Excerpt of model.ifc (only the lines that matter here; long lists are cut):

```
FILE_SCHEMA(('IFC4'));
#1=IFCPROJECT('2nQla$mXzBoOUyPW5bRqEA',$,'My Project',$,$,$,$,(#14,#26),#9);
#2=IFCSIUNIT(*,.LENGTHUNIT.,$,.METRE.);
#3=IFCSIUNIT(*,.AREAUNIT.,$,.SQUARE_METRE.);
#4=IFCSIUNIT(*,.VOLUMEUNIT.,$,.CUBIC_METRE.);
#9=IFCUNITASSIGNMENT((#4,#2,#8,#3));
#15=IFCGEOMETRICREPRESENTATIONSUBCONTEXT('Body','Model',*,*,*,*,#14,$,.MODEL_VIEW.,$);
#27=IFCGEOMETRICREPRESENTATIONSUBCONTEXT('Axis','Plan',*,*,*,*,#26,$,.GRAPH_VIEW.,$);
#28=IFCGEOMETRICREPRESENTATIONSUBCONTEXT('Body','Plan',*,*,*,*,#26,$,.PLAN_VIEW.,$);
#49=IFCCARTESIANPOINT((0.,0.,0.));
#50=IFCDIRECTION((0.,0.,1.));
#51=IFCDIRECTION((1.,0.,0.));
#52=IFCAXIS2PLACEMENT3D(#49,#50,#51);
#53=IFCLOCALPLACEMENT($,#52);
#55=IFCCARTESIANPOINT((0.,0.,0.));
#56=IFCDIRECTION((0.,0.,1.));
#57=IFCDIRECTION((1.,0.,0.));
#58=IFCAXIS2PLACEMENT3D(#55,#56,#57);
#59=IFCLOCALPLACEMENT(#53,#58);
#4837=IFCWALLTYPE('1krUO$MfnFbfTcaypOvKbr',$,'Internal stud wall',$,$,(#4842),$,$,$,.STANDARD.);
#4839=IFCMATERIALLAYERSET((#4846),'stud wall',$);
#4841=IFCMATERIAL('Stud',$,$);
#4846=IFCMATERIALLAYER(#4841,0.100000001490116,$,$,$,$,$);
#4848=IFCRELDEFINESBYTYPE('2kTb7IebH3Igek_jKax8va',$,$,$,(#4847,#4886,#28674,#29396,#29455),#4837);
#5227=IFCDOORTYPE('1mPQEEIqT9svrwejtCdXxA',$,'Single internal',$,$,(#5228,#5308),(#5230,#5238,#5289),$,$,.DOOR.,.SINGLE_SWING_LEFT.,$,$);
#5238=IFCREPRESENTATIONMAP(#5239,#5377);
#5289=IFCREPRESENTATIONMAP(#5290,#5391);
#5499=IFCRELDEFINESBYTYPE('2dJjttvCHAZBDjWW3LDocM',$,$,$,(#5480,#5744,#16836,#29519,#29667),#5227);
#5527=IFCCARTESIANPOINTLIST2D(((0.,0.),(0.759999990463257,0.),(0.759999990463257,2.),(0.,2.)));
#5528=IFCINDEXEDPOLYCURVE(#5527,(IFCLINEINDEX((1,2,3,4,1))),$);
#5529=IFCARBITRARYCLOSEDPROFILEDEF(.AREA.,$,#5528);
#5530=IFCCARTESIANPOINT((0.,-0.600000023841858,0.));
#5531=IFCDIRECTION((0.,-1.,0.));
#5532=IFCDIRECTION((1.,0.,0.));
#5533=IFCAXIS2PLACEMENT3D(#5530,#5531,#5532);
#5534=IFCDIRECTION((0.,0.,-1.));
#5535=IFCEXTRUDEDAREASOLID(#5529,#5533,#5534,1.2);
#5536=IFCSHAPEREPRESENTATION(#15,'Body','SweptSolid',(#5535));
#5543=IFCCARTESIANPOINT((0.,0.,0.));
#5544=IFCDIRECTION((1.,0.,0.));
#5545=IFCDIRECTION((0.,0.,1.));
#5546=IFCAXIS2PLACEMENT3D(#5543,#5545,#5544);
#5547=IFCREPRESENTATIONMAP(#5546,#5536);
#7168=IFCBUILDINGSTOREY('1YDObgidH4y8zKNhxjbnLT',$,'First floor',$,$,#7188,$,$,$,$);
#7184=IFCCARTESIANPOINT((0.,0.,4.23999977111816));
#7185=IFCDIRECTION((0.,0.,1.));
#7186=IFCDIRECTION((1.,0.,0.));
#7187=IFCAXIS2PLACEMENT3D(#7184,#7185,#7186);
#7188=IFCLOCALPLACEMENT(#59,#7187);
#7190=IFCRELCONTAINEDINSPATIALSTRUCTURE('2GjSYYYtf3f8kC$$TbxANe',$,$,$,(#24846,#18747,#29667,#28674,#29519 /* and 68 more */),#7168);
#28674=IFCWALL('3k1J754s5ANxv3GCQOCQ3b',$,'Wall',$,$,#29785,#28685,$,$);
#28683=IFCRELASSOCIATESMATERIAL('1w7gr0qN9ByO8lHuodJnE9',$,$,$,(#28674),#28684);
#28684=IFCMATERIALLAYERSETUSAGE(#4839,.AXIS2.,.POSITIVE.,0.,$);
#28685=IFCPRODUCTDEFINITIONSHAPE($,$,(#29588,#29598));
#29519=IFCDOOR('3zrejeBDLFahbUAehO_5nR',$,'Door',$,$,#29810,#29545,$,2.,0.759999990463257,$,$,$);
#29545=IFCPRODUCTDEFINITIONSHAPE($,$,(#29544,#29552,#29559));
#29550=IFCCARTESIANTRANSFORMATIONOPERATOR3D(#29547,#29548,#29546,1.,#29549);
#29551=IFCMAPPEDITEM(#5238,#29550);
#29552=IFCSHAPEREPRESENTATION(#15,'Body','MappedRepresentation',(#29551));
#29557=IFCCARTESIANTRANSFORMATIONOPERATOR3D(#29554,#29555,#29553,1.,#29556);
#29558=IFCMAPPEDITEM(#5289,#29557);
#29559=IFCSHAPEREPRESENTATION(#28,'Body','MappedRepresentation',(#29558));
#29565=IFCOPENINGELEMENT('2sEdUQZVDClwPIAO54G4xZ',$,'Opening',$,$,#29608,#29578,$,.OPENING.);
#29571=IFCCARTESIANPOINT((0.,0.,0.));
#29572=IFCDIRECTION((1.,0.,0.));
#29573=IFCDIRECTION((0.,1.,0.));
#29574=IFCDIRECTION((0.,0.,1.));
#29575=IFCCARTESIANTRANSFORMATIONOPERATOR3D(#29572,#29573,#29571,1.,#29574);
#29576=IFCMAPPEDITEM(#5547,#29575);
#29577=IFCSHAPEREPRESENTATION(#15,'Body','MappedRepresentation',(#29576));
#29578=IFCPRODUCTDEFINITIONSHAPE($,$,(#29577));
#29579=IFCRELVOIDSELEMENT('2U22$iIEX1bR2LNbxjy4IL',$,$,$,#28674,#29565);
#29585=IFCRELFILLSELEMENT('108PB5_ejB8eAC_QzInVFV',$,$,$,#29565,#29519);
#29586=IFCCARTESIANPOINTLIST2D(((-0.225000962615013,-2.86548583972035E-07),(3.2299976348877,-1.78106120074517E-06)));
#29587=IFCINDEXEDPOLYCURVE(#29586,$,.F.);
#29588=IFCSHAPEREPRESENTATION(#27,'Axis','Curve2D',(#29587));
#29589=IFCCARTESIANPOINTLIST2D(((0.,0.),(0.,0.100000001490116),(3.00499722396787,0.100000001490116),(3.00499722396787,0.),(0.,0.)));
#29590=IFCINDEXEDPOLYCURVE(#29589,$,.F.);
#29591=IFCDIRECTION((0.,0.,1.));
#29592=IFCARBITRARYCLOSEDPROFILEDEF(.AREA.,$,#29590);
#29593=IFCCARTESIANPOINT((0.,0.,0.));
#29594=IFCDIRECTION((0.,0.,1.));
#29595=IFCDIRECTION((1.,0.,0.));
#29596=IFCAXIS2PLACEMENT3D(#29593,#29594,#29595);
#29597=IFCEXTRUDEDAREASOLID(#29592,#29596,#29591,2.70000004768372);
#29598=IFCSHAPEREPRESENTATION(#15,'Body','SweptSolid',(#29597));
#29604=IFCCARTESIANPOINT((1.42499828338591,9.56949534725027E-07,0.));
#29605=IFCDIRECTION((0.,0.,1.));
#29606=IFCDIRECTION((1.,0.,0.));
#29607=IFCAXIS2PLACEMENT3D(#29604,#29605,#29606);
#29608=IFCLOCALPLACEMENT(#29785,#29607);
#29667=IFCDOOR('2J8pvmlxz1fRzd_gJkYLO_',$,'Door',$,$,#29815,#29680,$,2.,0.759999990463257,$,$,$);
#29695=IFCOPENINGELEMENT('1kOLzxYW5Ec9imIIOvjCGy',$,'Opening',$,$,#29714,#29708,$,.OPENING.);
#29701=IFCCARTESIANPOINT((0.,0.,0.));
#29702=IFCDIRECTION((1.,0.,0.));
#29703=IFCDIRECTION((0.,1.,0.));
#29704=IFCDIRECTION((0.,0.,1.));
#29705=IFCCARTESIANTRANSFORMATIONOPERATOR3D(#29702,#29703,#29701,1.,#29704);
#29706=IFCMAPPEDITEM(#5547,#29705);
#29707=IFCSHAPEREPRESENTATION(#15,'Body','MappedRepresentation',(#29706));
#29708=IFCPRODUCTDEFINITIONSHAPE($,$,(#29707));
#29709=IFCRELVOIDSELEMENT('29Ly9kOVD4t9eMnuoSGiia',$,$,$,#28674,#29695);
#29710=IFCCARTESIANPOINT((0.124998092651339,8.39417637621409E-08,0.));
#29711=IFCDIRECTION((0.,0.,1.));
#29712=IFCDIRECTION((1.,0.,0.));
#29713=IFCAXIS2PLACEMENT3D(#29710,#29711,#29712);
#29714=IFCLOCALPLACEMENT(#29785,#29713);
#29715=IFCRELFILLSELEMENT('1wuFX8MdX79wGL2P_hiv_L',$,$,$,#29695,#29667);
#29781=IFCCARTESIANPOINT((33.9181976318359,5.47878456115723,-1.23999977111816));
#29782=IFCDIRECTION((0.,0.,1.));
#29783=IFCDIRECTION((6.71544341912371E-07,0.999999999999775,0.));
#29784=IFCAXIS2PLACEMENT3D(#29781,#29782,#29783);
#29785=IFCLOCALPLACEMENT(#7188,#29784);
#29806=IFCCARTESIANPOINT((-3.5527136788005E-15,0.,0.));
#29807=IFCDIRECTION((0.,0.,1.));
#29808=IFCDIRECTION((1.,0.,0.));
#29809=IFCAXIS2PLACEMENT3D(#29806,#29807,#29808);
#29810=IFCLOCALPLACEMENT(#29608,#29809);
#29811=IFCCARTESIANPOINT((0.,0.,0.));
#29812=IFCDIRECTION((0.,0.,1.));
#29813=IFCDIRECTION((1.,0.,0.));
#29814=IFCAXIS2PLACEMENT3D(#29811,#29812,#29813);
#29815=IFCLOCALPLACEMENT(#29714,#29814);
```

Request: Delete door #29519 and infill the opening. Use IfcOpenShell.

```python
import ifcopenshell
import ifcopenshell.api.feature
import ifcopenshell.api.root
import ifcopenshell.geom
import ifcopenshell.util.shape

model = ifcopenshell.open("model.ifc")
settings = ifcopenshell.geom.settings()


def volume(element):
    """Net volume in cubic metres, openings subtracted."""
    shape = ifcopenshell.geom.create_shape(settings, element)
    return ifcopenshell.util.shape.get_volume(shape.geometry)


door = model.by_guid("3zrejeBDLFahbUAehO_5nR")
opening = door.FillsVoids[0].RelatingOpeningElement
wall = opening.VoidsElements[0].RelatingBuildingElement
before = volume(wall)

ifcopenshell.api.root.remove_product(model, product=door)
ifcopenshell.api.feature.remove_feature(model, feature=opening)

after = volume(wall)

print(f"wall volume {before:.3f} -> {after:.3f} m3")

model.write("model-out.ifc")
```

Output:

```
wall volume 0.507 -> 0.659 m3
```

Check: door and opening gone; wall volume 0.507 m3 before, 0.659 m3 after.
